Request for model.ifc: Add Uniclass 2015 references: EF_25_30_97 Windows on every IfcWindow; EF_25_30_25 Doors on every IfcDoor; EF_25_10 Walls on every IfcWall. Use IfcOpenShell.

First a look at what the model holds.

```python
import ifcopenshell

model = ifcopenshell.open("model.ifc")
print(model.schema)
print("classifications:", [c.Name for c in model.by_type("IfcClassification")])
for ifc_class in ("IfcDoor", "IfcRoof", "IfcStair", "IfcWall", "IfcWindow"):
    print(ifc_class, len(model.by_type(ifc_class)))
```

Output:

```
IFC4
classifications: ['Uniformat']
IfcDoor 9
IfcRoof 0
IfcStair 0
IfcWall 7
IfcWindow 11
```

```python
import ifcopenshell
import ifcopenshell.api.classification

model = ifcopenshell.open("model.ifc")

system = ifcopenshell.api.classification.add_classification(model, classification="Uniclass 2015")

codes = {
    "IfcWindow": ("EF_25_30_97", "Windows"),
    "IfcDoor": ("EF_25_30_25", "Doors"),
    "IfcWall": ("EF_25_10", "Walls"),
}
for ifc_class, (code, name) in codes.items():
    products = model.by_type(ifc_class)
    ifcopenshell.api.classification.add_reference(
        model, products=products, classification=system, identification=code, name=name
    )
    print(code, len(products))

model.write("model-out.ifc")
```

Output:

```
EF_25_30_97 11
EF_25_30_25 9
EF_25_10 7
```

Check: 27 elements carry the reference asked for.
